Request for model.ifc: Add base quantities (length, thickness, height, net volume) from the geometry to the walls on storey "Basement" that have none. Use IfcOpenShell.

First a look at what the model holds.

```python
import ifcopenshell
import ifcopenshell.util.element
import ifcopenshell.util.unit

model = ifcopenshell.open("model.ifc")
print(model.schema)
for unit_type in ("LENGTHUNIT", "AREAUNIT", "VOLUMEUNIT"):
    print(unit_type, ifcopenshell.util.unit.calculate_unit_scale(model, unit_type))
storey = next(s for s in model.by_type("IfcBuildingStorey") if s.Name == "Basement")
walls = [e for e in ifcopenshell.util.element.get_decomposition(storey) if e.is_a("IfcWall")]
for e in sorted(walls, key=lambda e: e.id()):
    print(e.id(), e.is_a(), e.Name, list(ifcopenshell.util.element.get_psets(e, qtos_only=True)), sep=" | ")
```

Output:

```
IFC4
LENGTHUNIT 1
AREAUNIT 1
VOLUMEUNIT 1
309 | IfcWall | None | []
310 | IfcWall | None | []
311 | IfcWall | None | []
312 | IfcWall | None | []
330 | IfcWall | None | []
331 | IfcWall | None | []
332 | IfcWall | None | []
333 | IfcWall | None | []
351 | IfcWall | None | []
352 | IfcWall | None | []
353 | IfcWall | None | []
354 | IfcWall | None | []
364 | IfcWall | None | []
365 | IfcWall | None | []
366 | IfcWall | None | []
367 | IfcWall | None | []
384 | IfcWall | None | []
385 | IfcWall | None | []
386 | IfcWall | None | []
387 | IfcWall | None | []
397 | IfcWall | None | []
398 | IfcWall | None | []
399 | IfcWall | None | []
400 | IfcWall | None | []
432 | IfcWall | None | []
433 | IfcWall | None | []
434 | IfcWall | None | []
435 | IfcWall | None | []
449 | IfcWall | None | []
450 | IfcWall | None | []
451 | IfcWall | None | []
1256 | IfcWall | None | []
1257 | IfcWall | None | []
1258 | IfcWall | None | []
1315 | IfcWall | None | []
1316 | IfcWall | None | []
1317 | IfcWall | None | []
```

```python
import ifcopenshell
import ifcopenshell.api.pset
import ifcopenshell.geom
import ifcopenshell.util.element
import ifcopenshell.util.shape
import ifcopenshell.util.unit

model = ifcopenshell.open("model.ifc")
unit_scale = ifcopenshell.util.unit.calculate_unit_scale(model)
volume_scale = ifcopenshell.util.unit.calculate_unit_scale(model, "VOLUMEUNIT")
settings = ifcopenshell.geom.settings()

storey = next(s for s in model.by_type("IfcBuildingStorey") if s.Name == "Basement")
walls = [e for e in ifcopenshell.util.element.get_decomposition(storey) if e.is_a("IfcWall")]

for e in sorted(walls, key=lambda e: e.id()):
    if ifcopenshell.util.element.get_psets(e, qtos_only=True, should_inherit=False):
        continue
    # Geometry comes back in metres, in the element's own axes.
    shape = ifcopenshell.geom.create_shape(settings, e)
    values = {
        "Length": ifcopenshell.util.shape.get_x(shape.geometry) / unit_scale,
        "Width": ifcopenshell.util.shape.get_y(shape.geometry) / unit_scale,
        "Height": ifcopenshell.util.shape.get_z(shape.geometry) / unit_scale,
        "NetVolume": ifcopenshell.util.shape.get_volume(shape.geometry) / volume_scale,
    }
    qto = ifcopenshell.api.pset.add_qto(model, product=e, name="Qto_WallBaseQuantities")
    ifcopenshell.api.pset.edit_qto(model, qto=qto, properties=values)
    print(e.id(), {k: round(v, 3) for k, v in values.items()})

model.write("model_rev.ifc")
```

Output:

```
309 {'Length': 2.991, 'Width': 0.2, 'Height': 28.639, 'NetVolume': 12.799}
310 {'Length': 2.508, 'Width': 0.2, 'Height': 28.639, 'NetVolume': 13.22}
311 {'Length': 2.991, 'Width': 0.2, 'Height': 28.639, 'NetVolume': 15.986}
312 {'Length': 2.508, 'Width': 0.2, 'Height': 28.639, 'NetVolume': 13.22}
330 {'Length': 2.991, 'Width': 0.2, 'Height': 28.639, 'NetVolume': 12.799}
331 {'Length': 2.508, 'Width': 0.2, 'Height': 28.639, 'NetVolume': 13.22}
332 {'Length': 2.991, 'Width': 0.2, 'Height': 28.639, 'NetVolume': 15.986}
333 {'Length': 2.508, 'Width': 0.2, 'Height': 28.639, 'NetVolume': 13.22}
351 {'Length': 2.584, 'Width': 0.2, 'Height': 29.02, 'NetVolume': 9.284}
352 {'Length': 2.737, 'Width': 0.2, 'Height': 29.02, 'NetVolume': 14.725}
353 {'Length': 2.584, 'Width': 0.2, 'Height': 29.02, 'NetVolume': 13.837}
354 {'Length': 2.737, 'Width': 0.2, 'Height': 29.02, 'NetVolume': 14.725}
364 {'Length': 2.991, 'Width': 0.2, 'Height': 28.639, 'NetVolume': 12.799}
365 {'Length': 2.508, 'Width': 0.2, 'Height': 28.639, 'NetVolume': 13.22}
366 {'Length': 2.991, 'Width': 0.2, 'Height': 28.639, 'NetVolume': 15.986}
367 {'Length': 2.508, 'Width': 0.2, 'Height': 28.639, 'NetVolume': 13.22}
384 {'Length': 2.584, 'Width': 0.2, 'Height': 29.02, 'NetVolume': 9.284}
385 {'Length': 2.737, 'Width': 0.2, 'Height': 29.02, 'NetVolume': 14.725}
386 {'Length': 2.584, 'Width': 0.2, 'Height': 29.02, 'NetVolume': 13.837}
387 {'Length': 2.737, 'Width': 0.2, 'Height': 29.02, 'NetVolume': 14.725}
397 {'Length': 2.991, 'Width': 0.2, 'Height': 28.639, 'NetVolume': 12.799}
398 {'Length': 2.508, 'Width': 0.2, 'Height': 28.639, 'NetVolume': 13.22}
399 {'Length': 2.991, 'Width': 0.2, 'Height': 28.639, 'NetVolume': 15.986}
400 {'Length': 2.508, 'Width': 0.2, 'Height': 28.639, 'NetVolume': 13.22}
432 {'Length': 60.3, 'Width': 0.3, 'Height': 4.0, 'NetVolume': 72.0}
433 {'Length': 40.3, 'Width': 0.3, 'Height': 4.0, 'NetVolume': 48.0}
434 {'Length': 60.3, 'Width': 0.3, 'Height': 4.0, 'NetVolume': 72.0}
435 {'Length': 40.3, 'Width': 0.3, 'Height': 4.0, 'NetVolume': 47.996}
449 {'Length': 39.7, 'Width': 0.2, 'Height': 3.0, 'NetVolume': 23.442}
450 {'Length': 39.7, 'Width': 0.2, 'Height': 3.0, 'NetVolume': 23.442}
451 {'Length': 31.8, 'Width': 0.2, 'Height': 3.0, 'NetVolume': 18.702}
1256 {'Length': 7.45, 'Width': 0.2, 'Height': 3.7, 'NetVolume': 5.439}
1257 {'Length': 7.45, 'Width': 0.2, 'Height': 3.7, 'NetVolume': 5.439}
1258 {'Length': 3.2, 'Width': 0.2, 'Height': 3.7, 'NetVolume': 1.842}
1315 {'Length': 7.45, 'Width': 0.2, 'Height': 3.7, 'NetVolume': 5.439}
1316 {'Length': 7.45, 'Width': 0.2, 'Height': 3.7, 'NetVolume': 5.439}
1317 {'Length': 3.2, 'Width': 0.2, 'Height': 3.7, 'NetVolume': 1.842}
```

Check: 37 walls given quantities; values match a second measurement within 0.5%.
